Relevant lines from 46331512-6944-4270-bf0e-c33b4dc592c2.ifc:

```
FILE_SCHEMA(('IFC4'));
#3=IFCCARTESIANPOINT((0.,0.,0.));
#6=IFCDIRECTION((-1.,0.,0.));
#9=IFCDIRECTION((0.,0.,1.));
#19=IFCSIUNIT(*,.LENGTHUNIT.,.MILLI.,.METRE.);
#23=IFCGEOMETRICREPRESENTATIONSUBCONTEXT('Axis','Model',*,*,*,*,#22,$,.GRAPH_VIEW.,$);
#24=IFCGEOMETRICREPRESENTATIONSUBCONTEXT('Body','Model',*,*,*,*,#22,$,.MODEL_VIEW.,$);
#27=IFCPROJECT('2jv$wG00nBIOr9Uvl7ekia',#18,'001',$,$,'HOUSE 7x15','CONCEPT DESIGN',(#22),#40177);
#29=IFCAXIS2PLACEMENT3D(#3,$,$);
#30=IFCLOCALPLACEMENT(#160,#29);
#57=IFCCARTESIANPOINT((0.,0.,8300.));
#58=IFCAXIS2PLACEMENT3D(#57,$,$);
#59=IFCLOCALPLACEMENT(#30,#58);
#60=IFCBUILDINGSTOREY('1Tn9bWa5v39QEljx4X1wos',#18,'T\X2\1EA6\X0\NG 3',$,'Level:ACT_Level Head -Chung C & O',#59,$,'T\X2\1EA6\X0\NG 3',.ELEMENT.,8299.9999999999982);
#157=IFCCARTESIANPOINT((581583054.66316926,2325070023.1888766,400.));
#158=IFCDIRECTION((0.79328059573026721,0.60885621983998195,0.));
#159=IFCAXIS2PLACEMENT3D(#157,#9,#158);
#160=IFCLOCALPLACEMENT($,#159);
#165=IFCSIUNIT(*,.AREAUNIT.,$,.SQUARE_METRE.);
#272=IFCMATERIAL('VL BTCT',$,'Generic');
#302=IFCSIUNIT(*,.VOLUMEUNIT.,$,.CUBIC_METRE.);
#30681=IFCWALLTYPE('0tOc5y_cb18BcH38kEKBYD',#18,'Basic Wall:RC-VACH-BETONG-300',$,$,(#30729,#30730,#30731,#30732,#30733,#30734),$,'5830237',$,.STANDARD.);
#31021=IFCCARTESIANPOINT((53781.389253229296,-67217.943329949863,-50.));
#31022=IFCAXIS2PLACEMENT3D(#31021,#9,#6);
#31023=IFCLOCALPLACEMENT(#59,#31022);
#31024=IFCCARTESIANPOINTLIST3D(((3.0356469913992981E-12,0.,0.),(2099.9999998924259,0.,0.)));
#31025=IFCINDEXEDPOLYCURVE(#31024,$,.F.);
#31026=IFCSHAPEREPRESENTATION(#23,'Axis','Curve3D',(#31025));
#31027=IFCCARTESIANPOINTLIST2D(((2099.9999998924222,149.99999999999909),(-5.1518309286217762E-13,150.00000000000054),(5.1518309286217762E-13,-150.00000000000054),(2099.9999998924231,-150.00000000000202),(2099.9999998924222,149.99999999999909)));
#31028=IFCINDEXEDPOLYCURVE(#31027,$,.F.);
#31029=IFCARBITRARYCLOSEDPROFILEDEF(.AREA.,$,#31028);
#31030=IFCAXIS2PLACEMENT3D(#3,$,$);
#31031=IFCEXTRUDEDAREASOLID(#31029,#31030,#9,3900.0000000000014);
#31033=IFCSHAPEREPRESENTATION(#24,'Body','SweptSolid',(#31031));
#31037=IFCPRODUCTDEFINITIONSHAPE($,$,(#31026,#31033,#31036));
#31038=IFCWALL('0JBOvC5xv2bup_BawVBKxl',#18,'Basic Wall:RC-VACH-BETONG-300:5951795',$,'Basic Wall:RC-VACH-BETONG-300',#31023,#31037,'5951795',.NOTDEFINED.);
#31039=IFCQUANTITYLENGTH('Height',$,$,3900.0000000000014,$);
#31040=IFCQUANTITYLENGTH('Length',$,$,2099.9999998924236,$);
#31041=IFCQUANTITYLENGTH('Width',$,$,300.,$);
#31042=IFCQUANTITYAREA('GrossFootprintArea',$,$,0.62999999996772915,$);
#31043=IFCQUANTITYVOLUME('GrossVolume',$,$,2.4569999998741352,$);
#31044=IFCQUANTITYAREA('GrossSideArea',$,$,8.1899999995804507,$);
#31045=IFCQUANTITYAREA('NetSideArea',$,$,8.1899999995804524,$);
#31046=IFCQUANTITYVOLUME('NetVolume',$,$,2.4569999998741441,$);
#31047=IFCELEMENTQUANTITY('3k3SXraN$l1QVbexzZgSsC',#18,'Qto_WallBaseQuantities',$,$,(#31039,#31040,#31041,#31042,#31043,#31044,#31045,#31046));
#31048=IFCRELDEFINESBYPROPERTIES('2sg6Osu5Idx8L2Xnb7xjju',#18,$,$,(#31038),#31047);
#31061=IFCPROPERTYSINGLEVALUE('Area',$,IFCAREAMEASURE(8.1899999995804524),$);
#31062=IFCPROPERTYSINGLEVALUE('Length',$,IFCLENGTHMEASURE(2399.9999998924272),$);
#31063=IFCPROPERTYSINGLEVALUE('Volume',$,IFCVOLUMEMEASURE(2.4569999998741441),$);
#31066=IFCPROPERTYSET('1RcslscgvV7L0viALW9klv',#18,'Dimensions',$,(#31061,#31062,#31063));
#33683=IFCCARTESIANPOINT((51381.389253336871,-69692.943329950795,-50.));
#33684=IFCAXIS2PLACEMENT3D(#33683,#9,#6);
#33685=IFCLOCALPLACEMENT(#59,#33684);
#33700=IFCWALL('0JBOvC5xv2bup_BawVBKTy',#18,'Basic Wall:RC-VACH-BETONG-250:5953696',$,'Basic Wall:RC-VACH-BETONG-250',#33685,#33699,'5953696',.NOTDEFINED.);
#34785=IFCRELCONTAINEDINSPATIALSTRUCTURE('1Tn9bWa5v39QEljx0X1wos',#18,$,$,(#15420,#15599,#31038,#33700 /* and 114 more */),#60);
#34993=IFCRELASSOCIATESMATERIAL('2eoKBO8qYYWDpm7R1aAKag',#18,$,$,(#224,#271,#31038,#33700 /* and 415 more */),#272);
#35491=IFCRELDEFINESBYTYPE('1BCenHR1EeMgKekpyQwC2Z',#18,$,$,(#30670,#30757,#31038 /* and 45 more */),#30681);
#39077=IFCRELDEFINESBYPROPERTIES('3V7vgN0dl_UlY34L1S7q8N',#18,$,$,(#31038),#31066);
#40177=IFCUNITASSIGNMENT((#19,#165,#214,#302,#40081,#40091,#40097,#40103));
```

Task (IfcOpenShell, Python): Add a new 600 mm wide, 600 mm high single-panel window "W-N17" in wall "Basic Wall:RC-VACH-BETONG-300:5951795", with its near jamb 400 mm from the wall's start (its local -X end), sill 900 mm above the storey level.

```python
import numpy as np
import ifcopenshell
import ifcopenshell.api.feature
import ifcopenshell.api.geometry
import ifcopenshell.api.pset
import ifcopenshell.api.root
import ifcopenshell.api.spatial
import ifcopenshell.geom
import ifcopenshell.util.element
import ifcopenshell.util.placement
import ifcopenshell.util.representation
import ifcopenshell.util.shape
import ifcopenshell.util.unit

model = ifcopenshell.open("46331512-6944-4270-bf0e-c33b4dc592c2.ifc")
unit_scale = ifcopenshell.util.unit.calculate_unit_scale(model)
area_scale = ifcopenshell.util.unit.calculate_unit_scale(model, "AREAUNIT")
volume_scale = ifcopenshell.util.unit.calculate_unit_scale(model, "VOLUMEUNIT")
settings = ifcopenshell.geom.settings()


def volume(element):
    """Net volume in cubic metres, openings subtracted."""
    shape = ifcopenshell.geom.create_shape(settings, element)
    return ifcopenshell.util.shape.get_volume(shape.geometry)


wall = model.by_guid("0JBOvC5xv2bup_BawVBKxl")
storey = ifcopenshell.util.element.get_container(wall, ifc_class="IfcBuildingStorey")
context = ifcopenshell.util.representation.get_context(model, "Model", "Body", "MODEL_VIEW")
before = volume(wall)

width, height, from_end, sill = 0.6, 0.6, 0.4, 0.9  # metres

# The wall runs along its own X axis, and the end named is its -X end.
wall_shape = ifcopenshell.geom.create_shape(settings, wall)
x, y, z = ifcopenshell.util.shape.get_vertices(wall_shape.geometry).T
start = x.min() + from_end
face, thickness = float(y.min()), float(y.max() - y.min())
wall_matrix = ifcopenshell.util.placement.get_local_placement(wall.ObjectPlacement)
level = ifcopenshell.util.placement.get_local_placement(storey.ObjectPlacement)[2, 3]


def in_wall(x, y):
    """Placement at x, y metres in the wall's axes, at sill height."""
    matrix = wall_matrix.copy()
    matrix[:, 3] = wall_matrix @ np.array([x / unit_scale, y / unit_scale, 0.0, 1.0])
    matrix[2, 3] = level + sill / unit_scale
    return matrix


# Opening: a box that overshoots both wall faces by 50 mm.
opening = ifcopenshell.api.root.create_entity(model, ifc_class="IfcOpeningElement", predefined_type="OPENING")
box = ifcopenshell.api.geometry.add_wall_representation(
    model, context=context, length=width, height=height, thickness=thickness + 0.1
)
ifcopenshell.api.geometry.assign_representation(model, product=opening, representation=box)
ifcopenshell.api.geometry.edit_object_placement(model, product=opening, matrix=in_wall(start, face - 0.05), is_si=False)
ifcopenshell.api.feature.add_feature(model, feature=opening, element=wall)

window = ifcopenshell.api.root.create_entity(model, ifc_class="IfcWindow", name="W-N17", predefined_type="WINDOW")
window.OverallWidth, window.OverallHeight = width / unit_scale, height / unit_scale
window.PartitioningType = "SINGLE_PANEL"
body = ifcopenshell.api.geometry.add_window_representation(
    model,
    context=context,
    overall_width=window.OverallWidth,
    overall_height=window.OverallHeight,
    partition_type="SINGLE_PANEL",
)
ifcopenshell.api.geometry.assign_representation(model, product=window, representation=body)
ifcopenshell.api.spatial.assign_container(model, products=[window], relating_structure=storey)
ifcopenshell.api.feature.add_filling(model, opening=opening, element=window)

# Centre the window in the wall's thickness.
ifcopenshell.api.geometry.edit_object_placement(model, product=window, matrix=in_wall(start, face), is_si=False)
window_shape = ifcopenshell.geom.create_shape(settings, window)
depth = ifcopenshell.util.shape.get_vertices(window_shape.geometry)[:, 1]
offset = face + thickness / 2 - (depth.min() + depth.max()) / 2
ifcopenshell.api.geometry.edit_object_placement(model, product=window, matrix=in_wall(start, offset), is_si=False)

after = volume(wall)

# Update the wall's stored quantities.
qto = model.by_id(ifcopenshell.util.element.get_pset(wall, "Qto_WallBaseQuantities", should_inherit=False)["id"])
ifcopenshell.api.pset.edit_qto(model, qto=qto, properties={
    "NetSideArea": after / thickness / area_scale,
    "NetVolume": after / volume_scale,
})
pset = model.by_id(ifcopenshell.util.element.get_pset(wall, "Dimensions", should_inherit=False)["id"])
ifcopenshell.api.pset.edit_pset(model, pset=pset, properties={
    "Area": model.create_entity("IfcAreaMeasure", after / thickness / area_scale),
    "Volume": model.create_entity("IfcVolumeMeasure", after / volume_scale),
})

print(f"wall volume {before:.3f} -> {after:.3f} m3")

model.write("46331512-6944-4270-bf0e-c33b4dc592c2-out.ifc")
```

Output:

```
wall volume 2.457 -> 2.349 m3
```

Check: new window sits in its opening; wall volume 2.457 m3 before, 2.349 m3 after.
